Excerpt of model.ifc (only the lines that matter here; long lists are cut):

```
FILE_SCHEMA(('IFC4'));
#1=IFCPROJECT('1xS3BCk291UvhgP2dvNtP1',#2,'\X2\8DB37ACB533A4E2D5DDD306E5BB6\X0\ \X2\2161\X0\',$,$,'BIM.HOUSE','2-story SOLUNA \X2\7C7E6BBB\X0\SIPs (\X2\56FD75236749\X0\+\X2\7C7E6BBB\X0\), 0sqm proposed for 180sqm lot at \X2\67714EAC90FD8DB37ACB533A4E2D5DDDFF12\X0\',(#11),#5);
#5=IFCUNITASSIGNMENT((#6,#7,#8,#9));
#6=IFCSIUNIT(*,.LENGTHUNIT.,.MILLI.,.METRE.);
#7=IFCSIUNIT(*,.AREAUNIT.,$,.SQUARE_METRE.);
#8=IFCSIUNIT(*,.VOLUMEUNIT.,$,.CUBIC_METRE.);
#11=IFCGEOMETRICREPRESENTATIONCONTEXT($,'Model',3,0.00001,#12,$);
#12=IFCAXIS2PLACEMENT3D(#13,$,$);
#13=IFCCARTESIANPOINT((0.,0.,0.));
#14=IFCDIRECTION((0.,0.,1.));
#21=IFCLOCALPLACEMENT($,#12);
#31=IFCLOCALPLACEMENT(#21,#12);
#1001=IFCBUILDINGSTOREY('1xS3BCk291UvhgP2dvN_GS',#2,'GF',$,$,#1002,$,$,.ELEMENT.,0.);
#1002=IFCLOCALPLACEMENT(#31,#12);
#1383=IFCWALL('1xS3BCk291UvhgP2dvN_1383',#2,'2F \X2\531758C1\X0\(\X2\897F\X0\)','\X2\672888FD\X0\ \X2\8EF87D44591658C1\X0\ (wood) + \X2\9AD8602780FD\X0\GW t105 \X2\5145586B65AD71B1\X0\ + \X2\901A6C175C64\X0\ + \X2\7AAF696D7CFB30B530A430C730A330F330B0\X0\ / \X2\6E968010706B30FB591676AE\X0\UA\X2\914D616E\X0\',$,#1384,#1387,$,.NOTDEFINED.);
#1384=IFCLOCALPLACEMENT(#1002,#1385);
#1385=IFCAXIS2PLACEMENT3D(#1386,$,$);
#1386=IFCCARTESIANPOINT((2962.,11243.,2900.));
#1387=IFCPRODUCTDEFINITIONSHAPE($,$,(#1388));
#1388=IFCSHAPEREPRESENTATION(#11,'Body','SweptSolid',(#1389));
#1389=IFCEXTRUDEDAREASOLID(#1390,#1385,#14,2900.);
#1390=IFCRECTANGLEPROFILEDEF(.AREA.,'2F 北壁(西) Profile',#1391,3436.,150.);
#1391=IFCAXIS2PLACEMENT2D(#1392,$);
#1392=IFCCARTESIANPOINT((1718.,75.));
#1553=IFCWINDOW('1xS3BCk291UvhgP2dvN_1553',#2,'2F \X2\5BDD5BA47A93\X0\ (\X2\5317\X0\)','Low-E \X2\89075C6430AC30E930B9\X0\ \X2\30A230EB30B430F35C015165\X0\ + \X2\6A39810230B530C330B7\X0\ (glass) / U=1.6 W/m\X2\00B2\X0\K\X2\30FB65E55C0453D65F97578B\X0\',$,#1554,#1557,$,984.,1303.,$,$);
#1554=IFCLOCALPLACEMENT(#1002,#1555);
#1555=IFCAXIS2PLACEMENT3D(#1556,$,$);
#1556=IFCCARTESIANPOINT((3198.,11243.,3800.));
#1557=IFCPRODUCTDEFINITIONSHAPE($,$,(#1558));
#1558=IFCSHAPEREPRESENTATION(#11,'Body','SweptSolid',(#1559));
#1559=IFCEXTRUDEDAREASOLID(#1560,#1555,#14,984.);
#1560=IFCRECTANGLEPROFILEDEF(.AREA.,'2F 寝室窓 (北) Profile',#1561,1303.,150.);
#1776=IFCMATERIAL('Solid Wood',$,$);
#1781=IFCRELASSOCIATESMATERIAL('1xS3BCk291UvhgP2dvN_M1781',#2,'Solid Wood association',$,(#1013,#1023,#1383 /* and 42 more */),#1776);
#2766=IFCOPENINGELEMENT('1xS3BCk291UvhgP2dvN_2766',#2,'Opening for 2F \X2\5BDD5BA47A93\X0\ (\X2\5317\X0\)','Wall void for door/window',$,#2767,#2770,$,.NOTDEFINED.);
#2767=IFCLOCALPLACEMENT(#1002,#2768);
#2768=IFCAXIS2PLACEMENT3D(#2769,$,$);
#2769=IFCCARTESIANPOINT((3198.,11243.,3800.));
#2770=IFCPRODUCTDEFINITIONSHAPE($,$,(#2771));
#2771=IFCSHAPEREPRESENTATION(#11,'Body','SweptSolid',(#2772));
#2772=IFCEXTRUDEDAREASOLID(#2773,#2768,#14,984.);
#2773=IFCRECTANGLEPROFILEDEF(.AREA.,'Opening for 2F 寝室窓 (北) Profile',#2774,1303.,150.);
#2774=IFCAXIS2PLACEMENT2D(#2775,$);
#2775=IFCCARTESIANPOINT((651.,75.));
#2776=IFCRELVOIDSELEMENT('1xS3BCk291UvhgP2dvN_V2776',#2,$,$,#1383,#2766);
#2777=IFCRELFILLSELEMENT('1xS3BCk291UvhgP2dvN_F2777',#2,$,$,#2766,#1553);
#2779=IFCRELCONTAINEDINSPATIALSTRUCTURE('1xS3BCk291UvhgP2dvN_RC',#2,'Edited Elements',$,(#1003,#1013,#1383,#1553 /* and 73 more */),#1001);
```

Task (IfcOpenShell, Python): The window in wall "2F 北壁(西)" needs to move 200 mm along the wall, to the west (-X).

```python
import ifcopenshell
import ifcopenshell.api.geometry
import ifcopenshell.util.placement
import ifcopenshell.util.unit

model = ifcopenshell.open("model.ifc")
unit_scale = ifcopenshell.util.unit.calculate_unit_scale(model)

window = model.by_guid("1xS3BCk291UvhgP2dvN_1553")
opening = window.FillsVoids[0].RelatingOpeningElement
wall = opening.VoidsElements[0].RelatingBuildingElement

wall_matrix = ifcopenshell.util.placement.get_local_placement(wall.ObjectPlacement)
shift = wall_matrix[:3, 0] * -0.2 / unit_scale
before = ifcopenshell.util.placement.get_local_placement(window.ObjectPlacement)[:3, 3].copy()

# The window is not placed relative to its opening, so move both.
for product in (opening, window):
    matrix = ifcopenshell.util.placement.get_local_placement(product.ObjectPlacement)
    matrix[:3, 3] += shift
    ifcopenshell.api.geometry.edit_object_placement(model, product=product, matrix=matrix, is_si=False)

after = ifcopenshell.util.placement.get_local_placement(window.ObjectPlacement)[:3, 3]
print("window moved by", (after - before).round(3) + 0.0)

model.write("model_rev.ifc")
```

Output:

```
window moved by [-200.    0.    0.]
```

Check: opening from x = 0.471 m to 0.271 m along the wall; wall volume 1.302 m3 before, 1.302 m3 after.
